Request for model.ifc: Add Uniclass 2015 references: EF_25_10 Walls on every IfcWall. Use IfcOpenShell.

First a look at what the model holds.

```python
import ifcopenshell

model = ifcopenshell.open("model.ifc")
print(model.schema)
print("classifications:", [c.Name for c in model.by_type("IfcClassification")])
for ifc_class in ("IfcDoor", "IfcRoof", "IfcStair", "IfcWall", "IfcWindow"):
    print(ifc_class, len(model.by_type(ifc_class)))
```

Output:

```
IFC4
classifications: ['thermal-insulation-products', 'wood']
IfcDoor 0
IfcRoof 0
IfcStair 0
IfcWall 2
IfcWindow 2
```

```python
import ifcopenshell
import ifcopenshell.api.classification

model = ifcopenshell.open("model.ifc")

system = ifcopenshell.api.classification.add_classification(model, classification="Uniclass 2015")

codes = {
    "IfcWall": ("EF_25_10", "Walls"),
}
for ifc_class, (code, name) in codes.items():
    products = model.by_type(ifc_class)
    ifcopenshell.api.classification.add_reference(
        model, products=products, classification=system, identification=code, name=name
    )
    print(code, len(products))

model.write("model_edited.ifc")
```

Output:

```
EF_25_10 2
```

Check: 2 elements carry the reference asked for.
